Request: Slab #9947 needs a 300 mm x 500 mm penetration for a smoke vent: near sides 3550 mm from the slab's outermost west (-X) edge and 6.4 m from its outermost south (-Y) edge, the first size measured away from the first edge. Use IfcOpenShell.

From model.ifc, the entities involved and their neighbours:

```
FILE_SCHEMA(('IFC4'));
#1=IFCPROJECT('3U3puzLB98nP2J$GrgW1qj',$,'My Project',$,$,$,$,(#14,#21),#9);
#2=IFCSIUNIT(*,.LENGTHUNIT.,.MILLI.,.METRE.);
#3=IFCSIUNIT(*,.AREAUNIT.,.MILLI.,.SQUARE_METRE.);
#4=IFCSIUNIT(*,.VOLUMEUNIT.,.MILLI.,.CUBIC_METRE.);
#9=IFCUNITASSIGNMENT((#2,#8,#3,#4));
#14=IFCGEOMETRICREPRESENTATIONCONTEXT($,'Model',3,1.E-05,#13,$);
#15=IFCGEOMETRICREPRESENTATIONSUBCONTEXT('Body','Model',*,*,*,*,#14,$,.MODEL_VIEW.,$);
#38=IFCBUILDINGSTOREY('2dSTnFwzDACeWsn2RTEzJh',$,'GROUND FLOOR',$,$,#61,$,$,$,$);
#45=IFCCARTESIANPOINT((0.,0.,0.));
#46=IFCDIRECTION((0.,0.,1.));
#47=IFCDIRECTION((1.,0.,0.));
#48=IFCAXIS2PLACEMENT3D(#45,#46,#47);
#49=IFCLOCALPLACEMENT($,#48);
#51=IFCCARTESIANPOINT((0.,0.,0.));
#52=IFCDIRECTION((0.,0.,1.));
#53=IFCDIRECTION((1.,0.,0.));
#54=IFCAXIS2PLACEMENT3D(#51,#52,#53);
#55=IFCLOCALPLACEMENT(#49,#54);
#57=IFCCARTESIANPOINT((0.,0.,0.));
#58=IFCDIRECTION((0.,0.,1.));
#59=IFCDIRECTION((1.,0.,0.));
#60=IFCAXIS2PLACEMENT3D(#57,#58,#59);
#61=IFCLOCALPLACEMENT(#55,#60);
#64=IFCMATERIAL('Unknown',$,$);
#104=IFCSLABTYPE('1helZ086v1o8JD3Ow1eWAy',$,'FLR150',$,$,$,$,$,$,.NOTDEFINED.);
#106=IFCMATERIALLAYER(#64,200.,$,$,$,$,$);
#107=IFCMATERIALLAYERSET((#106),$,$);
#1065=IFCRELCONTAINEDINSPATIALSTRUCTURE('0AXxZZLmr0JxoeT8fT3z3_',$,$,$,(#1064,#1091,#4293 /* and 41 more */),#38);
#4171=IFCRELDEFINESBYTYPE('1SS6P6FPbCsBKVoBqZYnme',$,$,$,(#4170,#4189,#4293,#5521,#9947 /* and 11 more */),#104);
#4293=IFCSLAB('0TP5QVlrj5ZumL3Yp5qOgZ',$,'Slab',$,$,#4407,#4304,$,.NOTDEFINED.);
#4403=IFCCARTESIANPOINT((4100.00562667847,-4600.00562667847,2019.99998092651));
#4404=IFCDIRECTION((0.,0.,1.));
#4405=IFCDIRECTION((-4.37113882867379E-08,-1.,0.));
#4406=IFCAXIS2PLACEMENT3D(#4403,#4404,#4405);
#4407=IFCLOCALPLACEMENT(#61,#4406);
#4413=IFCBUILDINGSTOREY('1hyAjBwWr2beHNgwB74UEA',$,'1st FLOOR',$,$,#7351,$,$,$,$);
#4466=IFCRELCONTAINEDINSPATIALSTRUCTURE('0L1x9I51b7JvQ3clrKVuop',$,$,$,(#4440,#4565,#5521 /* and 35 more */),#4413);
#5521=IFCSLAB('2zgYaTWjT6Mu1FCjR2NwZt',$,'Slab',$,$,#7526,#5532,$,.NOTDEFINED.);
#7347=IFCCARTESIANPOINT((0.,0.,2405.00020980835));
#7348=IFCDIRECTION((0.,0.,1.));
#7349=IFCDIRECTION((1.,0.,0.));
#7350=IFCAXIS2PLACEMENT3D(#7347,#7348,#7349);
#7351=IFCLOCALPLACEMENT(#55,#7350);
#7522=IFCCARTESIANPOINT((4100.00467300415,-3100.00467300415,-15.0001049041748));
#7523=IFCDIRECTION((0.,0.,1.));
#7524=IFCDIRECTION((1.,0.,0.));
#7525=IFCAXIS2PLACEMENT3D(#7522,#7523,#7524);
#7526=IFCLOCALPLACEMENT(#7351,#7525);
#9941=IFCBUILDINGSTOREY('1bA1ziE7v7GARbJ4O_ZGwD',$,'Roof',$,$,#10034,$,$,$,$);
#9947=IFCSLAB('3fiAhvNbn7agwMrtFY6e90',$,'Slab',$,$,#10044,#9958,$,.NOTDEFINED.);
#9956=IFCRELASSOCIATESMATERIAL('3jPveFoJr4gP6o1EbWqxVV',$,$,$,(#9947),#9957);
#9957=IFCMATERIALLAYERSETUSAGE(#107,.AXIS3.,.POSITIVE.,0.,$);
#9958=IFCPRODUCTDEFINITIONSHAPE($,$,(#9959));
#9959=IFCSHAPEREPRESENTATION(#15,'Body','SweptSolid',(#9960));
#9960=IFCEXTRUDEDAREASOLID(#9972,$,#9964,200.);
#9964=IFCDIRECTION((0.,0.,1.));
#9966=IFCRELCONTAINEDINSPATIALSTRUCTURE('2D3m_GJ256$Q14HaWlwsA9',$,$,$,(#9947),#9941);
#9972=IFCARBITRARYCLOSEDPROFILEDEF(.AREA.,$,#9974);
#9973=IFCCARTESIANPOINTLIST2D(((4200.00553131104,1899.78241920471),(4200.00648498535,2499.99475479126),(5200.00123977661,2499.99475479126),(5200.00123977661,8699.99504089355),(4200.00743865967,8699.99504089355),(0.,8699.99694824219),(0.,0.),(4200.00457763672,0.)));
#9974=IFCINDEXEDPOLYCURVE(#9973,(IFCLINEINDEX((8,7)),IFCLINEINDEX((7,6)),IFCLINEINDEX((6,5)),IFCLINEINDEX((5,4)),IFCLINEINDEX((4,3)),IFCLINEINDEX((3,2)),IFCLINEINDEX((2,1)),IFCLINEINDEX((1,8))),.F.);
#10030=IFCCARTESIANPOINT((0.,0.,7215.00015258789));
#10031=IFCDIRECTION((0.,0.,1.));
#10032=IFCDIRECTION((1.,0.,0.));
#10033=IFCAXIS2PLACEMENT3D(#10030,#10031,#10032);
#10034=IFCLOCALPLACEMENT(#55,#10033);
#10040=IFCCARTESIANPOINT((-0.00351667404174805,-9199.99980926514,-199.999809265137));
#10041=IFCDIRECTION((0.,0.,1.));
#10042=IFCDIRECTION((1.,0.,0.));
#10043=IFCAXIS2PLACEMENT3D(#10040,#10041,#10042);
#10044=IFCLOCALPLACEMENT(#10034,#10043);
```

```python
import numpy as np
import ifcopenshell
import ifcopenshell.api.feature
import ifcopenshell.api.geometry
import ifcopenshell.api.root
import ifcopenshell.geom
import ifcopenshell.util.placement
import ifcopenshell.util.representation
import ifcopenshell.util.shape
import ifcopenshell.util.unit

model = ifcopenshell.open("model.ifc")
unit_scale = ifcopenshell.util.unit.calculate_unit_scale(model)
settings = ifcopenshell.geom.settings()


def volume(element):
    """Net volume in cubic metres, openings subtracted."""
    shape = ifcopenshell.geom.create_shape(settings, element)
    return ifcopenshell.util.shape.get_volume(shape.geometry)


slab = model.by_guid("3fiAhvNbn7agwMrtFY6e90")
before = volume(slab)

# Extent in the slab's own axes, in metres. The edges named are its -X and -Y sides.
slab_shape = ifcopenshell.geom.create_shape(settings, slab)
vertices = ifcopenshell.util.shape.get_vertices(slab_shape.geometry)
x_min, y_min, bottom = vertices.min(axis=0)
top = vertices[:, 2].max()

opening = ifcopenshell.api.root.create_entity(model, ifc_class="IfcOpeningElement", name="Smoke vent opening", predefined_type="OPENING")
context = ifcopenshell.util.representation.get_context(model, "Model", "Body", "MODEL_VIEW")
width, depth = 0.3, 0.5
outline = [(0.0, 0.0), (width, 0.0), (width, depth), (0.0, depth), (0.0, 0.0)]
# Overshoot both faces by 50 mm so the cut is clean.
shape = ifcopenshell.api.geometry.add_slab_representation(
    model, context=context, depth=top - bottom + 0.1, polyline=outline
)
ifcopenshell.api.geometry.assign_representation(model, product=opening, representation=shape)

matrix = ifcopenshell.util.placement.get_local_placement(slab.ObjectPlacement)
matrix[:, 3] = matrix @ np.append(np.array([x_min + 3.55, y_min + 6.4, bottom - 0.05]) / unit_scale, 1.0)
ifcopenshell.api.geometry.edit_object_placement(model, product=opening, matrix=matrix, is_si=False)
ifcopenshell.api.feature.add_feature(model, feature=opening, element=slab)

after = volume(slab)

print(f"slab volume {before:.3f} -> {after:.3f} m3")

model.write("model_v2.ifc")
```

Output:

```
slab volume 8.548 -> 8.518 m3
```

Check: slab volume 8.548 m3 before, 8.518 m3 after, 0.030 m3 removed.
